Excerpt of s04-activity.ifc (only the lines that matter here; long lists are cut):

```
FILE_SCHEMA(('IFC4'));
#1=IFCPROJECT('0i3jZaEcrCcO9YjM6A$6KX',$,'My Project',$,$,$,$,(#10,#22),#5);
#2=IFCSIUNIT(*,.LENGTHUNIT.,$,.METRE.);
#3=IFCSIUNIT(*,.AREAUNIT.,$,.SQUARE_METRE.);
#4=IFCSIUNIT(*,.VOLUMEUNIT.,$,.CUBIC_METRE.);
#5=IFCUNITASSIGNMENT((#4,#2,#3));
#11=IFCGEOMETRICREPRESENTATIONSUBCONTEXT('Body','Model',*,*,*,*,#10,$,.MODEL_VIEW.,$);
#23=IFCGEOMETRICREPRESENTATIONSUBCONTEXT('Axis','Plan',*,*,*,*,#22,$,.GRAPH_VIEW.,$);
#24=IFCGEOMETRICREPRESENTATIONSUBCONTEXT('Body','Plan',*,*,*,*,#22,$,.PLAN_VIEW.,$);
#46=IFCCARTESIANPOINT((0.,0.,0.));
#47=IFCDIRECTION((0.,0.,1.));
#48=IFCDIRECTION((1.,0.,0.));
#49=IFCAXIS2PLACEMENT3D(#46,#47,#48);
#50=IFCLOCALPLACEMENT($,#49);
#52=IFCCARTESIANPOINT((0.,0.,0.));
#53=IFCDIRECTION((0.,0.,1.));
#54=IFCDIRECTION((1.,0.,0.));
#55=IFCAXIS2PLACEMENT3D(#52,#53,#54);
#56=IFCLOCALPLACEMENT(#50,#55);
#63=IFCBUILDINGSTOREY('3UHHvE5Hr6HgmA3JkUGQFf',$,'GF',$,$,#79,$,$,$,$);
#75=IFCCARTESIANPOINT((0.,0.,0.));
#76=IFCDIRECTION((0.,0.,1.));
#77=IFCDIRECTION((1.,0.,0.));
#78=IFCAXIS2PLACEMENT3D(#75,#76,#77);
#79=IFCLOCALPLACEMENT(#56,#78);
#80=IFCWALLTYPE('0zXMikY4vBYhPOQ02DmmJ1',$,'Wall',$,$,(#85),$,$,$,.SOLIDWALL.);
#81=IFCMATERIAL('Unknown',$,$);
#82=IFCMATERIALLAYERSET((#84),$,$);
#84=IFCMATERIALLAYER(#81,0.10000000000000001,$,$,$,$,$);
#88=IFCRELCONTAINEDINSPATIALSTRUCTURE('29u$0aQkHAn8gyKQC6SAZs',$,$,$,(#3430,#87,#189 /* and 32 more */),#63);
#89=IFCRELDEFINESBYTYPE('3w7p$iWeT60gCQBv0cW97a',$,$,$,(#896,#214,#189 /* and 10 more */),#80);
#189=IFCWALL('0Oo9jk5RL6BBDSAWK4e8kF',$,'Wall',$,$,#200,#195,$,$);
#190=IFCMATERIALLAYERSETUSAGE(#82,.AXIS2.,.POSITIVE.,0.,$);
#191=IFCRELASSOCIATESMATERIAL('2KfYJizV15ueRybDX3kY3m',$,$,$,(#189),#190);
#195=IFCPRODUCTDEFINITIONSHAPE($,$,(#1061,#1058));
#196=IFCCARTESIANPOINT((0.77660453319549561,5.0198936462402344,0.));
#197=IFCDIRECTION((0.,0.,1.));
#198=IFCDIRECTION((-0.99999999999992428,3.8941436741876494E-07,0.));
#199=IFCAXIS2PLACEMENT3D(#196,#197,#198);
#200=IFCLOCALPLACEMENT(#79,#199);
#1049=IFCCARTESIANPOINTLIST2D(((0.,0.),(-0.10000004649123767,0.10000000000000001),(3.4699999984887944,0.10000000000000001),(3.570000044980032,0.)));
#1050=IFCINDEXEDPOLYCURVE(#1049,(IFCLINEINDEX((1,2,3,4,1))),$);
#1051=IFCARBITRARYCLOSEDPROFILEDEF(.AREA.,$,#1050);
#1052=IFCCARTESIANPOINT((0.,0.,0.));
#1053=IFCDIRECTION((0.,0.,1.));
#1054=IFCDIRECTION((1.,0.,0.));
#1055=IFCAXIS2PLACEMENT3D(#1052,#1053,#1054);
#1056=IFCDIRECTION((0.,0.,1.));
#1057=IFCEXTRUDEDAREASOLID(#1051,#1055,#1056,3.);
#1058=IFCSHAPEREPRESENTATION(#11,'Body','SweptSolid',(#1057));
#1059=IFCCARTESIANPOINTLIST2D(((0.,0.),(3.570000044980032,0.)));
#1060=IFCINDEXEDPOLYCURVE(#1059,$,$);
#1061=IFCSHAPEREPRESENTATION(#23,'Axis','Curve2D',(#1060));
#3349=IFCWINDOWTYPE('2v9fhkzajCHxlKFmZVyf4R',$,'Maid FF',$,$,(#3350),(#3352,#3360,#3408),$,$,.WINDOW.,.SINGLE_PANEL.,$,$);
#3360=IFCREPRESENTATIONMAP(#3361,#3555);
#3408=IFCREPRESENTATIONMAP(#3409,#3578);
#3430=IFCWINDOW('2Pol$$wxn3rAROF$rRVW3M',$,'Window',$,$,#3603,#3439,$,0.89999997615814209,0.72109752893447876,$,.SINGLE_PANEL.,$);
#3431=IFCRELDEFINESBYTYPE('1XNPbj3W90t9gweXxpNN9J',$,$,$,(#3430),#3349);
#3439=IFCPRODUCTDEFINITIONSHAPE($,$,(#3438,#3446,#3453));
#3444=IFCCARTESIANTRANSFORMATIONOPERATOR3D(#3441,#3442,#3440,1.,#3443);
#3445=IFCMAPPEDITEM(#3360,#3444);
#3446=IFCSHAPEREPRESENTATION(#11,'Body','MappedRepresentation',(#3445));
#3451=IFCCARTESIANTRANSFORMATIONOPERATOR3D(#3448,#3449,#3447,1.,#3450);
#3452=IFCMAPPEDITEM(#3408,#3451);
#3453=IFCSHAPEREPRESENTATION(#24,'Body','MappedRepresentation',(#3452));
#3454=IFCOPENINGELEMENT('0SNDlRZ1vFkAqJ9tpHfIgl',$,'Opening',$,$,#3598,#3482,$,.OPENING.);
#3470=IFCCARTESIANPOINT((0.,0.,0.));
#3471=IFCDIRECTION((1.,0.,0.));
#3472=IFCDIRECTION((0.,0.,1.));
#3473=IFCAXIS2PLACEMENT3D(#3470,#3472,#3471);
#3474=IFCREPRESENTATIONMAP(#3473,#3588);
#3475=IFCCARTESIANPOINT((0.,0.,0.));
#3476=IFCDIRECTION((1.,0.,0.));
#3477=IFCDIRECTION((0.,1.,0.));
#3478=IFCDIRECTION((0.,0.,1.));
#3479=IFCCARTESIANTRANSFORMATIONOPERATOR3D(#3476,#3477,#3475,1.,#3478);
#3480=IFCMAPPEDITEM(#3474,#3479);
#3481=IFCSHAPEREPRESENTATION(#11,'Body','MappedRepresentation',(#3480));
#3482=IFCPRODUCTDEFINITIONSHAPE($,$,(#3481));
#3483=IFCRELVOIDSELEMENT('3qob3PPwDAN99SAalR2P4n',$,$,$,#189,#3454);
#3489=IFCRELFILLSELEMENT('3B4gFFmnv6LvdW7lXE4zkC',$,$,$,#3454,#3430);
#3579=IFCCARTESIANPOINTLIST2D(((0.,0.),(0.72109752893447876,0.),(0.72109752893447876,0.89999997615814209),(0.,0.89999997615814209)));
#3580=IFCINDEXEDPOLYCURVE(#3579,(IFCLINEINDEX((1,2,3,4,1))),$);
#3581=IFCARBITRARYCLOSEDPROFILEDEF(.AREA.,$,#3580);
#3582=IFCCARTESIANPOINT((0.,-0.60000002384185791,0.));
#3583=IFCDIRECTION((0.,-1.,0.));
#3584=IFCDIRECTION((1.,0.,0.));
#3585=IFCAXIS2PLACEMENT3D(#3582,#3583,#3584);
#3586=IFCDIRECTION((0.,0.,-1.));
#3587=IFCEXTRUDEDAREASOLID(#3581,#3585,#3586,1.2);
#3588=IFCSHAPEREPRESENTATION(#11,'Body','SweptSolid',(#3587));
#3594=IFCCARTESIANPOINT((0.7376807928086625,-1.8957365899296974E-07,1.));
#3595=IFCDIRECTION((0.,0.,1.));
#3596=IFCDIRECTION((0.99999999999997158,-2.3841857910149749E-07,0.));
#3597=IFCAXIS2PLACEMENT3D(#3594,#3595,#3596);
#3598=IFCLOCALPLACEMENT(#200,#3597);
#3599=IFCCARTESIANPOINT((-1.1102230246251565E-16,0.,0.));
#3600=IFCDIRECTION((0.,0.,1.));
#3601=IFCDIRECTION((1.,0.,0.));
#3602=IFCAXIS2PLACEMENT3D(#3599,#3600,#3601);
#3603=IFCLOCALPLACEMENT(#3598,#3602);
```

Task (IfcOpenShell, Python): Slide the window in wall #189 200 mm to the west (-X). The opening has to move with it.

```python
import ifcopenshell
import ifcopenshell.api.geometry
import ifcopenshell.util.placement
import ifcopenshell.util.unit

model = ifcopenshell.open("s04-activity.ifc")
unit_scale = ifcopenshell.util.unit.calculate_unit_scale(model)

window = model.by_guid("2Pol$$wxn3rAROF$rRVW3M")
opening = window.FillsVoids[0].RelatingOpeningElement
wall = opening.VoidsElements[0].RelatingBuildingElement

wall_matrix = ifcopenshell.util.placement.get_local_placement(wall.ObjectPlacement)
shift = wall_matrix[:3, 0] * 0.2 / unit_scale
before = ifcopenshell.util.placement.get_local_placement(window.ObjectPlacement)[:3, 3].copy()

# The window is placed relative to its opening, so it follows when the opening moves.
matrix = ifcopenshell.util.placement.get_local_placement(opening.ObjectPlacement)
matrix[:3, 3] += shift
ifcopenshell.api.geometry.edit_object_placement(
    model, product=opening, matrix=matrix, is_si=False, should_transform_children=True
)

after = ifcopenshell.util.placement.get_local_placement(window.ObjectPlacement)[:3, 3]
print("window moved by", (after - before).round(3) + 0.0)

model.write("s04-activity_updated.ifc")
```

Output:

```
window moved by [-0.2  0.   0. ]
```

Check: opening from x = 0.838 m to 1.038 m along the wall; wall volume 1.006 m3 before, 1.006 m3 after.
